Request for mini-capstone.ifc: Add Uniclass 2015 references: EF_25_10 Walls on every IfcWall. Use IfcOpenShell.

First a look at what the model holds.

```python
import ifcopenshell

model = ifcopenshell.open("mini-capstone.ifc")
print(model.schema)
print("classifications:", [c.Name for c in model.by_type("IfcClassification")])
for ifc_class in ("IfcDoor", "IfcRoof", "IfcStair", "IfcWall", "IfcWindow"):
    print(ifc_class, len(model.by_type(ifc_class)))
```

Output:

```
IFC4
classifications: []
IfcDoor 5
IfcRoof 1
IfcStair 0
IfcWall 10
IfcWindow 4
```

```python
import ifcopenshell
import ifcopenshell.api.classification

model = ifcopenshell.open("mini-capstone.ifc")

system = ifcopenshell.api.classification.add_classification(model, classification="Uniclass 2015")

codes = {
    "IfcWall": ("EF_25_10", "Walls"),
}
for ifc_class, (code, name) in codes.items():
    products = model.by_type(ifc_class)
    ifcopenshell.api.classification.add_reference(
        model, products=products, classification=system, identification=code, name=name
    )
    print(code, len(products))

model.write("mini-capstone-out.ifc")
```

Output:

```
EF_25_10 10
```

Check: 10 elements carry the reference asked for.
